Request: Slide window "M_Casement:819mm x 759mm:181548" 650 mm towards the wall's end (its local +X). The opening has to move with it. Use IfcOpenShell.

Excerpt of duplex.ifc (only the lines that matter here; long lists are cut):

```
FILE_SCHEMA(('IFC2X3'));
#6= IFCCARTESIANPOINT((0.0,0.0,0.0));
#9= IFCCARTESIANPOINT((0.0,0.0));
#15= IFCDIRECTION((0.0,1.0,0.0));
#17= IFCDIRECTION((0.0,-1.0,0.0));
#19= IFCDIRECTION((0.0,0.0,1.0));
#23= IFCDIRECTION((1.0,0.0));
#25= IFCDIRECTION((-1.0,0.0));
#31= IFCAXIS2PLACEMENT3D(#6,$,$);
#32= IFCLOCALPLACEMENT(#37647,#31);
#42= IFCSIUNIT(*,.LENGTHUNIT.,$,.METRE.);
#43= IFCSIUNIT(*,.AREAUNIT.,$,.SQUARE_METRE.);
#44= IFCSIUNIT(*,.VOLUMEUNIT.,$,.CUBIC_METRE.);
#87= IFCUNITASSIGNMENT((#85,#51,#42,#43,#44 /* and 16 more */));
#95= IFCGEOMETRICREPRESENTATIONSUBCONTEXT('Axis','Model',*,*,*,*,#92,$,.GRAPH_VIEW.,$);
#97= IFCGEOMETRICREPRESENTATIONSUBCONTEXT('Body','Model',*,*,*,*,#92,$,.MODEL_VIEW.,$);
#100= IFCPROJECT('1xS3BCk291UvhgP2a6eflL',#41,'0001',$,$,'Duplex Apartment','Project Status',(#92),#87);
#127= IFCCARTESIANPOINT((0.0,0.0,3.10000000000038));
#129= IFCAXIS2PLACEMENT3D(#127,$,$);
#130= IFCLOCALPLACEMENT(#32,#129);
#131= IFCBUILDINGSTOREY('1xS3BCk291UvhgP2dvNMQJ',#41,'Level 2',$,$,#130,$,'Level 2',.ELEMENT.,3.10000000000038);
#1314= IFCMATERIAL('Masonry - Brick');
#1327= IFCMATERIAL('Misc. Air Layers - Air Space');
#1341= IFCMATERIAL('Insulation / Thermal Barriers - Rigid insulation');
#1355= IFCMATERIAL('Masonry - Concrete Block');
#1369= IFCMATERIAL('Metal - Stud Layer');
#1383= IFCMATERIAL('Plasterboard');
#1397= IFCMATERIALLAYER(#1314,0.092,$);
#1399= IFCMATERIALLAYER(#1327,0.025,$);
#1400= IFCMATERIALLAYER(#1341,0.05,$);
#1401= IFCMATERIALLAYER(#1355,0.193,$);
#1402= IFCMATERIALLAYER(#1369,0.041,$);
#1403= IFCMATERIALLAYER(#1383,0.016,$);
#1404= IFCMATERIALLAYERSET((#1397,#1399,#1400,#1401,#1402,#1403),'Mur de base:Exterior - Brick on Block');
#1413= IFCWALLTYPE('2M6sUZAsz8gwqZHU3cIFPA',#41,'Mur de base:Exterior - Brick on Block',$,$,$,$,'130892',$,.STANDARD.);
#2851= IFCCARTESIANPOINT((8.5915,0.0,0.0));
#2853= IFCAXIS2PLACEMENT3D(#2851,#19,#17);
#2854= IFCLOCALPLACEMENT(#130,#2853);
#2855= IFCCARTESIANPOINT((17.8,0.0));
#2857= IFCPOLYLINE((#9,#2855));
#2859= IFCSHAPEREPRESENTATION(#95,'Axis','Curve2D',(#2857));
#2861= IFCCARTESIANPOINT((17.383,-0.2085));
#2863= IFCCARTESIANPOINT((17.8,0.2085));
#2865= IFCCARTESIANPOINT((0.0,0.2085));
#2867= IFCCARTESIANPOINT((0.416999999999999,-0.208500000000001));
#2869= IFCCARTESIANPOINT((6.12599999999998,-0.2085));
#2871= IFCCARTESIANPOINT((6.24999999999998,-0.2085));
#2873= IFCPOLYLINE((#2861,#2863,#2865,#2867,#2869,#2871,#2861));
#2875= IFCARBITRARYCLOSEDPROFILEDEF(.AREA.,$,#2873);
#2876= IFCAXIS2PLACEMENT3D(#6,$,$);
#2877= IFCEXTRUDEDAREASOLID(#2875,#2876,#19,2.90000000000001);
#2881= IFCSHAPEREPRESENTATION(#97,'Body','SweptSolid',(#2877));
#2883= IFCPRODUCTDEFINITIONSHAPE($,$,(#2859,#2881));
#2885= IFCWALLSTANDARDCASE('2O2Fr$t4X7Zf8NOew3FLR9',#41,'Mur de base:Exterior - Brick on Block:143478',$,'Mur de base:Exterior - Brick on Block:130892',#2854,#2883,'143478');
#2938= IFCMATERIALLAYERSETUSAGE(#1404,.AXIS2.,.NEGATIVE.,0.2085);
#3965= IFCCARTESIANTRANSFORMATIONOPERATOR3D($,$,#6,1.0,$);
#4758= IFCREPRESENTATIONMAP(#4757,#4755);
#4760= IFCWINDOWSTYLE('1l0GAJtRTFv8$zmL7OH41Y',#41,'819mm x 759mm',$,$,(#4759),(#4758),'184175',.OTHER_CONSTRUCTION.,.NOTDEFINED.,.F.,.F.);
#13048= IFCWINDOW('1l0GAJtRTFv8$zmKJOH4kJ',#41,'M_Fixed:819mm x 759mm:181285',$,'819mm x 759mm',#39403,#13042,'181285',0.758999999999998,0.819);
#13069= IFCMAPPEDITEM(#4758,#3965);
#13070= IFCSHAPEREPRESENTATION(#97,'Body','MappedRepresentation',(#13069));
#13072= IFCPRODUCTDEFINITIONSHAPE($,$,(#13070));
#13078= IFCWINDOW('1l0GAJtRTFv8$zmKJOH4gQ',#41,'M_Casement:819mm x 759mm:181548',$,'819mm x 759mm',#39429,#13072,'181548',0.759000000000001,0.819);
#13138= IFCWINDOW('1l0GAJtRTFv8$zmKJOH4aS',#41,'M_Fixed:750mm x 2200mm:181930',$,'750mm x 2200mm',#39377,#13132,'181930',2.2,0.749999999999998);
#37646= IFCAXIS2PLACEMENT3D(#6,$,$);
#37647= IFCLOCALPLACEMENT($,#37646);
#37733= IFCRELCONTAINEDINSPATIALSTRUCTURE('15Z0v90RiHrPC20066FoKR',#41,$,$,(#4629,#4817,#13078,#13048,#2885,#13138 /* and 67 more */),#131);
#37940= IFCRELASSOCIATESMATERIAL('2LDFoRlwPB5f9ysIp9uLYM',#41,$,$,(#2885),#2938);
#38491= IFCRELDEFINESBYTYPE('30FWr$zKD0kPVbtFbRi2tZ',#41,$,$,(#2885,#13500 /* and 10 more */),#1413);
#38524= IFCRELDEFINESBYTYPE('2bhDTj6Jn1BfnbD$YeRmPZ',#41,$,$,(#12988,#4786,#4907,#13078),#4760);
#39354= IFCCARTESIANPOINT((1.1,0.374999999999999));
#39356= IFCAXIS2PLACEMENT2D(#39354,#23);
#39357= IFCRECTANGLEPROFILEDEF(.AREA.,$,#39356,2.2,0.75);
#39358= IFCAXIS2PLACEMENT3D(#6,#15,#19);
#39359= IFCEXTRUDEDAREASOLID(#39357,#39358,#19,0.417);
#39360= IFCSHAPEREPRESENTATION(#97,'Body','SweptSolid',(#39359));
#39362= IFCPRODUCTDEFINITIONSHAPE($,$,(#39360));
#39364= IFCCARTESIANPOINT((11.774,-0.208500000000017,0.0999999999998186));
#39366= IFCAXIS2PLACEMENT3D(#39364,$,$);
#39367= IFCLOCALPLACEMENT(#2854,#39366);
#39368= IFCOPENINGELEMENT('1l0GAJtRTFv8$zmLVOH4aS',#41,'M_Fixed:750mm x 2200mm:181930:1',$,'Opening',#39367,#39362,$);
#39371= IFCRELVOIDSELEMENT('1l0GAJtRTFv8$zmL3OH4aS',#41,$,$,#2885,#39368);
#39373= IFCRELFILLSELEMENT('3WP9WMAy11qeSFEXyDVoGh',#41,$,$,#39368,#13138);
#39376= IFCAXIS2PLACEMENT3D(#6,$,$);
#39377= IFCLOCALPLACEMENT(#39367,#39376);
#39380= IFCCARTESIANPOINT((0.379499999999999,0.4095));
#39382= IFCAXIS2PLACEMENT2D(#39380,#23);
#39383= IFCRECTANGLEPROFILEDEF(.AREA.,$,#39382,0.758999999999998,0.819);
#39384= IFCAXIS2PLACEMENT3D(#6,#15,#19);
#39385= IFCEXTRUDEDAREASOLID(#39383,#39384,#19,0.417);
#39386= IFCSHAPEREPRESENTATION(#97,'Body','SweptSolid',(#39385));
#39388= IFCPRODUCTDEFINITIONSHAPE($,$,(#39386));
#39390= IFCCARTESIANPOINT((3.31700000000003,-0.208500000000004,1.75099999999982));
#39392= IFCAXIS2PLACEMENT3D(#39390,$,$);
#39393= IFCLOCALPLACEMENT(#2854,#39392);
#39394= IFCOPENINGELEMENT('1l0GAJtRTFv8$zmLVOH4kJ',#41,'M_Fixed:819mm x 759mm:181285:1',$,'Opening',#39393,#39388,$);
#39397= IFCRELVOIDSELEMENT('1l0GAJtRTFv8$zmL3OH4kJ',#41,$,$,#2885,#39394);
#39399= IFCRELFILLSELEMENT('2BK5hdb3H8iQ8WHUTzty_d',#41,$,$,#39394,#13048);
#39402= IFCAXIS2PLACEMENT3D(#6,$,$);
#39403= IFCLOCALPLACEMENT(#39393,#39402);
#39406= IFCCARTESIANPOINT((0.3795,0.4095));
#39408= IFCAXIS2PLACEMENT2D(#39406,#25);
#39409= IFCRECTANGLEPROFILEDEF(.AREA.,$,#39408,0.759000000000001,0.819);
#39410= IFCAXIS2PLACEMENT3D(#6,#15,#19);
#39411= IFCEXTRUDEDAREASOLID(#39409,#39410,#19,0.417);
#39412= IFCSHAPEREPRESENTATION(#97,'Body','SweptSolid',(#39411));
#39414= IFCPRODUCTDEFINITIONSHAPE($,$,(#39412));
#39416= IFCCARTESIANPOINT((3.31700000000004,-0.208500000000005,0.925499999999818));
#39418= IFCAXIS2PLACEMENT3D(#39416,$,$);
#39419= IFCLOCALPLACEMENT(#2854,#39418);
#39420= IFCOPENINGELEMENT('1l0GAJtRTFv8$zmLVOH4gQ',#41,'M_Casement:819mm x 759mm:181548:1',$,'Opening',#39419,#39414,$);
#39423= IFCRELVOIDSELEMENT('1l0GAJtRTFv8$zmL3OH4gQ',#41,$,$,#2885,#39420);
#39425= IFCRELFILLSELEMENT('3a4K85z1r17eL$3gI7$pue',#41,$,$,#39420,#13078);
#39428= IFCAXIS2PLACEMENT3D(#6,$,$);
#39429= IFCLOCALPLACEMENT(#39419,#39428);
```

```python
import ifcopenshell
import ifcopenshell.api.geometry
import ifcopenshell.util.placement

model = ifcopenshell.open("duplex.ifc")

window = model.by_guid("1l0GAJtRTFv8$zmKJOH4gQ")
opening = window.FillsVoids[0].RelatingOpeningElement
wall = opening.VoidsElements[0].RelatingBuildingElement

wall_matrix = ifcopenshell.util.placement.get_local_placement(wall.ObjectPlacement)
shift = wall_matrix[:3, 0] * 0.65
before = ifcopenshell.util.placement.get_local_placement(window.ObjectPlacement)[:3, 3].copy()

# The window is placed relative to its opening, so it follows when the opening moves.
matrix = ifcopenshell.util.placement.get_local_placement(opening.ObjectPlacement)
matrix[:3, 3] += shift
ifcopenshell.api.geometry.edit_object_placement(
    model, product=opening, matrix=matrix, is_si=False, should_transform_children=True
)

after = ifcopenshell.util.placement.get_local_placement(window.ObjectPlacement)[:3, 3]
print("window moved by", (after - before).round(3) + 0.0)

model.write("duplex-out.ifc")
```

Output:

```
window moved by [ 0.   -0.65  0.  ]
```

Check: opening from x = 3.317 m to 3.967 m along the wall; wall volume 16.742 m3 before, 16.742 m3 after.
